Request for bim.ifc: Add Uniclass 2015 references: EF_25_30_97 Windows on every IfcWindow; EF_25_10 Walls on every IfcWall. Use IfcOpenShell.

First a look at what the model holds.

```python
import ifcopenshell

model = ifcopenshell.open("bim.ifc")
print(model.schema)
print("classifications:", [c.Name for c in model.by_type("IfcClassification")])
for ifc_class in ("IfcDoor", "IfcRoof", "IfcStair", "IfcWall", "IfcWindow"):
    print(ifc_class, len(model.by_type(ifc_class)))
```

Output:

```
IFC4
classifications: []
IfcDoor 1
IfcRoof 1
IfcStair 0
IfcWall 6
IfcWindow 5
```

```python
import ifcopenshell
import ifcopenshell.api.classification

model = ifcopenshell.open("bim.ifc")

system = ifcopenshell.api.classification.add_classification(model, classification="Uniclass 2015")

codes = {
    "IfcWindow": ("EF_25_30_97", "Windows"),
    "IfcWall": ("EF_25_10", "Walls"),
}
for ifc_class, (code, name) in codes.items():
    products = model.by_type(ifc_class)
    ifcopenshell.api.classification.add_reference(
        model, products=products, classification=system, identification=code, name=name
    )
    print(code, len(products))

model.write("bim_updated.ifc")
```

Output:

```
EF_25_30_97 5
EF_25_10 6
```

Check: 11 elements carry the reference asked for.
